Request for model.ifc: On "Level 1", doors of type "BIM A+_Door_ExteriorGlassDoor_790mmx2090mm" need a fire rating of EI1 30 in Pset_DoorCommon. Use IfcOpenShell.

First a look at what the model holds.

```python
import ifcopenshell
import ifcopenshell.util.element

model = ifcopenshell.open("model.ifc")
print(model.schema)
storey = next(s for s in model.by_type("IfcBuildingStorey") if s.Name == "Level 1")
doors = [e for e in ifcopenshell.util.element.get_decomposition(storey) if e.is_a("IfcDoor")]
seen = {}
for e in doors:
    element_type = ifcopenshell.util.element.get_type(e)
    key = (element_type.Name if element_type != e and element_type else None, ifcopenshell.util.element.get_pset(e, "Pset_DoorCommon", "FireRating"))
    seen[key] = seen.get(key, 0) + 1
for (name, value), count in sorted(seen.items(), key=str):
    print(count, "x", name, "|", value)
```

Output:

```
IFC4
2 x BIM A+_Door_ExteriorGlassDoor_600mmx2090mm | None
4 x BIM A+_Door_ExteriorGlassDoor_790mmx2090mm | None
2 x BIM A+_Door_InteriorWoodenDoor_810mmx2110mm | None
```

```python
import ifcopenshell
import ifcopenshell.api.pset
import ifcopenshell.util.element

model = ifcopenshell.open("model.ifc")

storey = next(s for s in model.by_type("IfcBuildingStorey") if s.Name == "Level 1")
doors = [e for e in ifcopenshell.util.element.get_decomposition(storey) if e.is_a("IfcDoor")]

count = 0
for e in doors:
    element_type = ifcopenshell.util.element.get_type(e)
    if element_type in (None, e) or element_type.Name != "BIM A+_Door_ExteriorGlassDoor_790mmx2090mm":
        continue
    # add_pset returns the element's existing set when there is one.
    pset = ifcopenshell.api.pset.add_pset(model, product=e, name="Pset_DoorCommon")
    ifcopenshell.api.pset.edit_pset(model, pset=pset, properties={"FireRating": "EI1 30"})
    count += 1

print(count, "doors updated")

model.write("model_edited.ifc")
```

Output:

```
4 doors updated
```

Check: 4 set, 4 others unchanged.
